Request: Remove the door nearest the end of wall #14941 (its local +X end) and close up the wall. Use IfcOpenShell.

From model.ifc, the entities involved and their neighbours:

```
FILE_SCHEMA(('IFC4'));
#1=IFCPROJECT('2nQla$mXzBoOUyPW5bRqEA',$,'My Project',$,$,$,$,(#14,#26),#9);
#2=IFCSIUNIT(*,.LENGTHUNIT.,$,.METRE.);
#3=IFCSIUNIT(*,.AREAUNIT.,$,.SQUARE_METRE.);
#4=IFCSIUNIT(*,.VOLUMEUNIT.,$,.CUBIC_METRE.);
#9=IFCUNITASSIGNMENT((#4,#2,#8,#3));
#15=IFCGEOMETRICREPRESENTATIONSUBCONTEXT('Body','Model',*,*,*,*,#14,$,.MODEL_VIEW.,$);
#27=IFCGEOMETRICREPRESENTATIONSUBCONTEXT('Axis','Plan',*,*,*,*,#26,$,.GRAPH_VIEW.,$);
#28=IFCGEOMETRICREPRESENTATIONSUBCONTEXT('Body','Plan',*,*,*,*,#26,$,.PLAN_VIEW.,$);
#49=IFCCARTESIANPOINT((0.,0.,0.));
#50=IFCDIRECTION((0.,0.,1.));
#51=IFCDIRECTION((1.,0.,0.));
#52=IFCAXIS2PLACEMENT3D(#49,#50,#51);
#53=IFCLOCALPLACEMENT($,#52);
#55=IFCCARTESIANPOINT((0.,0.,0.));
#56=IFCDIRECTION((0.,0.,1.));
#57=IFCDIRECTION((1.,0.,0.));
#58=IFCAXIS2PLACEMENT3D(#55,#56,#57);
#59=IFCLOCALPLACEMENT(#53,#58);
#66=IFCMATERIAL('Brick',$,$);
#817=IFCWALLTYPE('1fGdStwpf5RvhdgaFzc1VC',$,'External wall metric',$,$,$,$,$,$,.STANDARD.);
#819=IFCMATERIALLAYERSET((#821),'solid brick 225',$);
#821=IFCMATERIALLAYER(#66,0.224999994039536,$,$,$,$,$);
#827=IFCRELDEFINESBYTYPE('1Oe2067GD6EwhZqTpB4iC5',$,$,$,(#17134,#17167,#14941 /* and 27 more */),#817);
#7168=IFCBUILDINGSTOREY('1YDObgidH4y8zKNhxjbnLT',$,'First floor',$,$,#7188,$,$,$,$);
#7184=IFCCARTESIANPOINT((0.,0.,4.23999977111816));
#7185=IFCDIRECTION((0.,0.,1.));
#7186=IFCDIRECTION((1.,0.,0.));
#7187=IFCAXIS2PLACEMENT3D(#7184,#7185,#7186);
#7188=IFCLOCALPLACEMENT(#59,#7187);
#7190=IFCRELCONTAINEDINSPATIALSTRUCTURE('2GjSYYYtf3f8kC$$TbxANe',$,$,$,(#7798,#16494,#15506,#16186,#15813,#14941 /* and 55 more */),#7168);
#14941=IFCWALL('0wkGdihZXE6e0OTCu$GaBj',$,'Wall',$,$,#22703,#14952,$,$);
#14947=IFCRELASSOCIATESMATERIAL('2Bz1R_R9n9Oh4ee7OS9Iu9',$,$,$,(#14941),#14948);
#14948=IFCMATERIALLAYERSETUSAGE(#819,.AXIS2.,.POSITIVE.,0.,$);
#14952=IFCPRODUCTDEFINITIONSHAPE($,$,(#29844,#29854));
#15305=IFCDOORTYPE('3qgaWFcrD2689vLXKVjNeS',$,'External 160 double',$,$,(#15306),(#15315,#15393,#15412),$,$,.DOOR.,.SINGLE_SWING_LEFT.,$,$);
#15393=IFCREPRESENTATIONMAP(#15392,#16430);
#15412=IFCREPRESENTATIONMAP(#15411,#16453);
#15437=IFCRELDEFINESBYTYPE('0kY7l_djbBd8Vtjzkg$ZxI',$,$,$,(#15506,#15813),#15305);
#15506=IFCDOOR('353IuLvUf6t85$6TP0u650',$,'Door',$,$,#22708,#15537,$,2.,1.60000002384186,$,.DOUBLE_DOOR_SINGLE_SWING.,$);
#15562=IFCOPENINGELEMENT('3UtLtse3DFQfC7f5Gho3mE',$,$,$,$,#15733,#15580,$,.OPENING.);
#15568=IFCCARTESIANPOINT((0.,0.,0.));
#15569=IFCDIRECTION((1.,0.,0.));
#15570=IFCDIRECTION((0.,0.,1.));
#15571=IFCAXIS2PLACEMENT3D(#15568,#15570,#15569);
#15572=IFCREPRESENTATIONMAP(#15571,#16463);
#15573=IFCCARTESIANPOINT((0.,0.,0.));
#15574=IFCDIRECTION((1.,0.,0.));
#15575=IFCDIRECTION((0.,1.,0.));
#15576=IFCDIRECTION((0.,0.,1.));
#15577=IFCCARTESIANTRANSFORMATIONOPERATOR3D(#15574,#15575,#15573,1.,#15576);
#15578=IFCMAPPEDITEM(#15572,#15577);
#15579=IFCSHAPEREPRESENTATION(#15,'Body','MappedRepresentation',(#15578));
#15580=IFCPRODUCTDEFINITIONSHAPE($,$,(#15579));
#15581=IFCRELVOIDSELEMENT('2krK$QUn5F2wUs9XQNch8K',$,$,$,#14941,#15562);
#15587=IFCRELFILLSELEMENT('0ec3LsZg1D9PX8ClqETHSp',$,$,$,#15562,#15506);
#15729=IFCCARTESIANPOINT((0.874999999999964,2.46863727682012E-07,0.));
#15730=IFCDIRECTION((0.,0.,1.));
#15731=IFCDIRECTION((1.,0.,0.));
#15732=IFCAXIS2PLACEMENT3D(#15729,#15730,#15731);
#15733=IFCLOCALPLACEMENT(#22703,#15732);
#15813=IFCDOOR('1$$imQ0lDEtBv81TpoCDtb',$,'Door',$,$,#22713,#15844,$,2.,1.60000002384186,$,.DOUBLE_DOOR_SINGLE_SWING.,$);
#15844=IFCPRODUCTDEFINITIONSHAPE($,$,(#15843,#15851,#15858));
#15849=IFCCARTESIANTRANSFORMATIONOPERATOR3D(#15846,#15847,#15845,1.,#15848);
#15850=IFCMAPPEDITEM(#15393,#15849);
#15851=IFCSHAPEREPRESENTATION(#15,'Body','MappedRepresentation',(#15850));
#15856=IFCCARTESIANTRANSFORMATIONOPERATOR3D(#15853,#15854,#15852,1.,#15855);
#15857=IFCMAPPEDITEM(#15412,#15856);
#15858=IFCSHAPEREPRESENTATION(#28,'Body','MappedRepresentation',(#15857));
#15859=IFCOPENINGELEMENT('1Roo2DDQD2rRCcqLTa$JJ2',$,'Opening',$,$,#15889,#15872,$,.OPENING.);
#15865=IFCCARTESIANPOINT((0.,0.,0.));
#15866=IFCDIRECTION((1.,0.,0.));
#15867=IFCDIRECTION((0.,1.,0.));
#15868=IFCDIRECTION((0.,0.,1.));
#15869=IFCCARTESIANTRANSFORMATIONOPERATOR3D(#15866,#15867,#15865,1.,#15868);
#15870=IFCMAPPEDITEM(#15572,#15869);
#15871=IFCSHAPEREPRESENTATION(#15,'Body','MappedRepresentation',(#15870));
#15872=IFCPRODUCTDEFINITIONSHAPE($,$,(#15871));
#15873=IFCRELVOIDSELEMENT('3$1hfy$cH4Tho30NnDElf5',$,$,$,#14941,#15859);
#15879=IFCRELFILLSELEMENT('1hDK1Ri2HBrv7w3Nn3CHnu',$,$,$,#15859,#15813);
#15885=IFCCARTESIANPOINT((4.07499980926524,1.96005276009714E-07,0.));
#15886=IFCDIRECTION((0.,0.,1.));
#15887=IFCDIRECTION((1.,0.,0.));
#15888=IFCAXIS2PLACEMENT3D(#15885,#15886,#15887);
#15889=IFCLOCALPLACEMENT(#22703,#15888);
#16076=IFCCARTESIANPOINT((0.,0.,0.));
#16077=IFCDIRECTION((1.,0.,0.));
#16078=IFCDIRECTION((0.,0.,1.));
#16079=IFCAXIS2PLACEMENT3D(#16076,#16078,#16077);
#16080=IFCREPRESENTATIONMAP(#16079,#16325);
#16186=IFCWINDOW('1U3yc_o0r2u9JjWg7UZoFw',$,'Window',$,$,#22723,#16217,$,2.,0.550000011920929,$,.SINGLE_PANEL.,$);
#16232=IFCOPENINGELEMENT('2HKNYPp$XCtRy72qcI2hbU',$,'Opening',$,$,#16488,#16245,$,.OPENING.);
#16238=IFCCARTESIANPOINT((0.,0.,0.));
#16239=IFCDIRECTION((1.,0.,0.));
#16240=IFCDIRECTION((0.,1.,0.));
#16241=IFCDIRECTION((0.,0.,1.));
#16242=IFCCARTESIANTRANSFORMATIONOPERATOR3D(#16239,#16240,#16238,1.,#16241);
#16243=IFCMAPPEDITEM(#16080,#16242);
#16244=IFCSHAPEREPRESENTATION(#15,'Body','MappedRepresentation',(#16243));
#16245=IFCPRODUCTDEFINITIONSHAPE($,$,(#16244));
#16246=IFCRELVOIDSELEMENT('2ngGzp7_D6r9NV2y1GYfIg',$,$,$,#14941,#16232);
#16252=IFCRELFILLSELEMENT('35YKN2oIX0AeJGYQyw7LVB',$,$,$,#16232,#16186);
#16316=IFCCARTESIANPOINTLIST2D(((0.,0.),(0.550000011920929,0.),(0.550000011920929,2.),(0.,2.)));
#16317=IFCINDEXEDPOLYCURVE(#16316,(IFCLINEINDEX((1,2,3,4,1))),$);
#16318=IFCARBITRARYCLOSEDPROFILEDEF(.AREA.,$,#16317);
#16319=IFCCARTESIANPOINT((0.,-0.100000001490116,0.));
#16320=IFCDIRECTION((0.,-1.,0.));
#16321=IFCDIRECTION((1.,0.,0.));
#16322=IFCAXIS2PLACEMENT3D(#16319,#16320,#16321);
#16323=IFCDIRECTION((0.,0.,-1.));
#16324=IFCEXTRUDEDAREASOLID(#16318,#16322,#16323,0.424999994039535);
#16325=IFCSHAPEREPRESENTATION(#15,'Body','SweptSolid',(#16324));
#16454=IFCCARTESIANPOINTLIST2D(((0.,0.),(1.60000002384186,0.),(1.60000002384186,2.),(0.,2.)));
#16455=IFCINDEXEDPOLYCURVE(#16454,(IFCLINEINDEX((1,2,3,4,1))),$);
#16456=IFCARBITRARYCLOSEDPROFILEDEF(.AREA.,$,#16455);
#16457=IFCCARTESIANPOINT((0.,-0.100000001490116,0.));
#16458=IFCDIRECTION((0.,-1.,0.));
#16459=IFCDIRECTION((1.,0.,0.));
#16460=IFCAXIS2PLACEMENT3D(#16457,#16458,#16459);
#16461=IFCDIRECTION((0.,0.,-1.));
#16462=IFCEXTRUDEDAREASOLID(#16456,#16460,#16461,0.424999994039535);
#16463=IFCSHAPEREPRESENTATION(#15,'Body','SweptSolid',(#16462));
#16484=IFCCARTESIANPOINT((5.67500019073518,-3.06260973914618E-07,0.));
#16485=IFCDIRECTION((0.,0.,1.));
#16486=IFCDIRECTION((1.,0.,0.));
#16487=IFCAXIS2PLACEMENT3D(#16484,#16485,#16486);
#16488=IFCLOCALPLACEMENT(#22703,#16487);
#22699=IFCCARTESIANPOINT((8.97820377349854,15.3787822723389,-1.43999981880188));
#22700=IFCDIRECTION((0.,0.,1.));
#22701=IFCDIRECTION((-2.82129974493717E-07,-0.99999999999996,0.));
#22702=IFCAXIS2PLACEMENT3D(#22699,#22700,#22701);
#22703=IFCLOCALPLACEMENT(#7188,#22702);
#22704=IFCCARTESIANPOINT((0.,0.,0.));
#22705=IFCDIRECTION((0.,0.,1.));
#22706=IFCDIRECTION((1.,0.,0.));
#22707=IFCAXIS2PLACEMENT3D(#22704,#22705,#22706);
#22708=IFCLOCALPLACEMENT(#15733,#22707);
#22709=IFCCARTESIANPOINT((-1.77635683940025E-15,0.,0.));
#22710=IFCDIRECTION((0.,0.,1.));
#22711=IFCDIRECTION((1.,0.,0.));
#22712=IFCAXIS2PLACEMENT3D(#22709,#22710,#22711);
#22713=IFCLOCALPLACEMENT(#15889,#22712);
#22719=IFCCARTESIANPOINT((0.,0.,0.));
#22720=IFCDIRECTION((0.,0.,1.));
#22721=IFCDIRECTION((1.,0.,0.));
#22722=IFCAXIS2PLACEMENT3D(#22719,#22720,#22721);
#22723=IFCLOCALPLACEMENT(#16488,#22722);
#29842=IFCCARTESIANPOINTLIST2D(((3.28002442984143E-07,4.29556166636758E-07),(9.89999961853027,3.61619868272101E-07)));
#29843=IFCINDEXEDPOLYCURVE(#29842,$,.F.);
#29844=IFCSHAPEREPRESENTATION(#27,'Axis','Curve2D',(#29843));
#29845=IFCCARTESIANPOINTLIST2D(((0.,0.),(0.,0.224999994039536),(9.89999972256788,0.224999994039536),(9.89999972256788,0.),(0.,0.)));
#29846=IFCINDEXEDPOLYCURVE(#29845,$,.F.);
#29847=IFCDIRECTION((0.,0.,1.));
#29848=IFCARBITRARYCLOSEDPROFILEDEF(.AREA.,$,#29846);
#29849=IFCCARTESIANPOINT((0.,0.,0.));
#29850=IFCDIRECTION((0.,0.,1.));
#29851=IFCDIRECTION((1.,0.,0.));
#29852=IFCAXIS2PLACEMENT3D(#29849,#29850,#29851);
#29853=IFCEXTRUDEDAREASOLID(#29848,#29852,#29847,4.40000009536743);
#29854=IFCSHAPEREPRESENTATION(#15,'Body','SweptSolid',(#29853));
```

```python
import ifcopenshell
import ifcopenshell.api.feature
import ifcopenshell.api.root
import ifcopenshell.geom
import ifcopenshell.util.shape

model = ifcopenshell.open("model.ifc")
settings = ifcopenshell.geom.settings()


def volume(element):
    """Net volume in cubic metres, openings subtracted."""
    shape = ifcopenshell.geom.create_shape(settings, element)
    return ifcopenshell.util.shape.get_volume(shape.geometry)


door = model.by_id(15813)
opening = door.FillsVoids[0].RelatingOpeningElement
wall = opening.VoidsElements[0].RelatingBuildingElement
before = volume(wall)

ifcopenshell.api.root.remove_product(model, product=door)
ifcopenshell.api.feature.remove_feature(model, feature=opening)

after = volume(wall)

print(f"wall volume {before:.3f} -> {after:.3f} m3")

model.write("model-out.ifc")
```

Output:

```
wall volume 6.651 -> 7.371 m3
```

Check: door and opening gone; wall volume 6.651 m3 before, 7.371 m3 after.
